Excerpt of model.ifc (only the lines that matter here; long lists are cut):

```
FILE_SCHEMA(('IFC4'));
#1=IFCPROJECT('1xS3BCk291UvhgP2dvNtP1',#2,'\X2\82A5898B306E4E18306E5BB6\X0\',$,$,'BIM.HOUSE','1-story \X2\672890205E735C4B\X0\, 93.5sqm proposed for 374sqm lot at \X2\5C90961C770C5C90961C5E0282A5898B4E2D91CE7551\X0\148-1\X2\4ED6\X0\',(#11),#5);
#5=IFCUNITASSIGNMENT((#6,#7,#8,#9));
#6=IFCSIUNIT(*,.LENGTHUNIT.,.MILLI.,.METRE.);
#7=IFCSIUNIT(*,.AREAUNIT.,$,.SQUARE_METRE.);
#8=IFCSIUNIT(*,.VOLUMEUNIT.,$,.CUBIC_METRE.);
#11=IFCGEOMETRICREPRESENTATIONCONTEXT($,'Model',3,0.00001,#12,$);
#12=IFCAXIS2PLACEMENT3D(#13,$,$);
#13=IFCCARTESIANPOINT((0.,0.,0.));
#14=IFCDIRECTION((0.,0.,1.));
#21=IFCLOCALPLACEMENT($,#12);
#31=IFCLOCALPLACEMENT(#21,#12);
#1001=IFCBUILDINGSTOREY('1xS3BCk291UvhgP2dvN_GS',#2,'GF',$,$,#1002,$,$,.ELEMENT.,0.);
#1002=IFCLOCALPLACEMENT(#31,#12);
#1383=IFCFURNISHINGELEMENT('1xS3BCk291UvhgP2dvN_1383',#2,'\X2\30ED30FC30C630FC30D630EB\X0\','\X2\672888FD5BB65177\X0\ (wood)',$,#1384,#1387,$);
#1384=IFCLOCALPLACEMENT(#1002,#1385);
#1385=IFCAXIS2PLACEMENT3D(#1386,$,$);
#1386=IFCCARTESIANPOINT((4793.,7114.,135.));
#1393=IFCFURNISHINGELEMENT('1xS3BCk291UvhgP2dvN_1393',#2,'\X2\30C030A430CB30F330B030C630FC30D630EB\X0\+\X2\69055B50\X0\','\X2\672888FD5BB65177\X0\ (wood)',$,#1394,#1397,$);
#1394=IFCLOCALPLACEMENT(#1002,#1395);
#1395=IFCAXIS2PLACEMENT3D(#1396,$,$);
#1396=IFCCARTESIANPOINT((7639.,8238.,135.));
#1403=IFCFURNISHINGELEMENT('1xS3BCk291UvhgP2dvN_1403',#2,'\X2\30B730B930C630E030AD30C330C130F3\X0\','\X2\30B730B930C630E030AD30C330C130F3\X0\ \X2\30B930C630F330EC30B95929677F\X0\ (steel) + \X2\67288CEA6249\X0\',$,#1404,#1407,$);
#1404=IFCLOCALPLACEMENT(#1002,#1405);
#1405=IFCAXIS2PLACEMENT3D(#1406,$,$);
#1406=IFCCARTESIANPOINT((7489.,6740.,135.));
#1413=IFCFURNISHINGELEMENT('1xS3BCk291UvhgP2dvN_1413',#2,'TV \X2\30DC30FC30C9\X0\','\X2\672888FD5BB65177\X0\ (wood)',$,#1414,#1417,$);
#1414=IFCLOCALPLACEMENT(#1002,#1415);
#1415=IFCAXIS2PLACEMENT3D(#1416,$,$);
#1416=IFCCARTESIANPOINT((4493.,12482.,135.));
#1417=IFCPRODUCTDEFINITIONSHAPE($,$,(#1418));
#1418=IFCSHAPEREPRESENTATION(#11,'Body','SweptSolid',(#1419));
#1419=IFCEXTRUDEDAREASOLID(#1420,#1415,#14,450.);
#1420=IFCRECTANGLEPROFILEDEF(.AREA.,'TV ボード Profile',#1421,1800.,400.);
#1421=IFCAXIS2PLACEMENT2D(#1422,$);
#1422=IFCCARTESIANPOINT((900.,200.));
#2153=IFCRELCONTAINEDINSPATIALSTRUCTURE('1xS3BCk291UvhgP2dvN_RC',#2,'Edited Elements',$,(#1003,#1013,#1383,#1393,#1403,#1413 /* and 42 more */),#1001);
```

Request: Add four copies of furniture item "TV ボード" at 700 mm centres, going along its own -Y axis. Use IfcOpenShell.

```python
import ifcopenshell
import ifcopenshell.api.geometry
import ifcopenshell.api.root
import ifcopenshell.util.element
import ifcopenshell.util.placement
import ifcopenshell.util.unit

model = ifcopenshell.open("model.ifc")
unit_scale = ifcopenshell.util.unit.calculate_unit_scale(model)


def reuse_history(source, copy):
    """copy_class also copies each property set's owner history, people and application; keep the originals."""
    for rel in copy.IsDefinedBy:
        if rel.is_a("IfcRelDefinesByProperties") and (history := rel.RelatingPropertyDefinition.OwnerHistory):
            rel.RelatingPropertyDefinition.OwnerHistory = source.OwnerHistory
            ifcopenshell.util.element.remove_deep2(model, history)


source = model.by_guid("1xS3BCk291UvhgP2dvN_1413")
base = ifcopenshell.util.placement.get_local_placement(source.ObjectPlacement)
step = -base[:3, 1] * 0.7 / unit_scale

for i in range(1, 5):
    copy = ifcopenshell.api.root.copy_class(model, product=source)
    copy.Representation = ifcopenshell.util.element.copy_deep(
        model, source.Representation, exclude=["IfcGeometricRepresentationContext", "IfcRepresentationMap"]
    )
    reuse_history(source, copy)
    matrix = base.copy()
    matrix[:3, 3] += i * step
    print("added at", matrix[:3, 3].round(3) + 0.0)
    ifcopenshell.api.geometry.edit_object_placement(model, product=copy, matrix=matrix, is_si=False)

model.write("model-out.ifc")
```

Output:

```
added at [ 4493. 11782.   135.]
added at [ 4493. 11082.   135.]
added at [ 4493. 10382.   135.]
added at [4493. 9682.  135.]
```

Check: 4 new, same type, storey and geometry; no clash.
